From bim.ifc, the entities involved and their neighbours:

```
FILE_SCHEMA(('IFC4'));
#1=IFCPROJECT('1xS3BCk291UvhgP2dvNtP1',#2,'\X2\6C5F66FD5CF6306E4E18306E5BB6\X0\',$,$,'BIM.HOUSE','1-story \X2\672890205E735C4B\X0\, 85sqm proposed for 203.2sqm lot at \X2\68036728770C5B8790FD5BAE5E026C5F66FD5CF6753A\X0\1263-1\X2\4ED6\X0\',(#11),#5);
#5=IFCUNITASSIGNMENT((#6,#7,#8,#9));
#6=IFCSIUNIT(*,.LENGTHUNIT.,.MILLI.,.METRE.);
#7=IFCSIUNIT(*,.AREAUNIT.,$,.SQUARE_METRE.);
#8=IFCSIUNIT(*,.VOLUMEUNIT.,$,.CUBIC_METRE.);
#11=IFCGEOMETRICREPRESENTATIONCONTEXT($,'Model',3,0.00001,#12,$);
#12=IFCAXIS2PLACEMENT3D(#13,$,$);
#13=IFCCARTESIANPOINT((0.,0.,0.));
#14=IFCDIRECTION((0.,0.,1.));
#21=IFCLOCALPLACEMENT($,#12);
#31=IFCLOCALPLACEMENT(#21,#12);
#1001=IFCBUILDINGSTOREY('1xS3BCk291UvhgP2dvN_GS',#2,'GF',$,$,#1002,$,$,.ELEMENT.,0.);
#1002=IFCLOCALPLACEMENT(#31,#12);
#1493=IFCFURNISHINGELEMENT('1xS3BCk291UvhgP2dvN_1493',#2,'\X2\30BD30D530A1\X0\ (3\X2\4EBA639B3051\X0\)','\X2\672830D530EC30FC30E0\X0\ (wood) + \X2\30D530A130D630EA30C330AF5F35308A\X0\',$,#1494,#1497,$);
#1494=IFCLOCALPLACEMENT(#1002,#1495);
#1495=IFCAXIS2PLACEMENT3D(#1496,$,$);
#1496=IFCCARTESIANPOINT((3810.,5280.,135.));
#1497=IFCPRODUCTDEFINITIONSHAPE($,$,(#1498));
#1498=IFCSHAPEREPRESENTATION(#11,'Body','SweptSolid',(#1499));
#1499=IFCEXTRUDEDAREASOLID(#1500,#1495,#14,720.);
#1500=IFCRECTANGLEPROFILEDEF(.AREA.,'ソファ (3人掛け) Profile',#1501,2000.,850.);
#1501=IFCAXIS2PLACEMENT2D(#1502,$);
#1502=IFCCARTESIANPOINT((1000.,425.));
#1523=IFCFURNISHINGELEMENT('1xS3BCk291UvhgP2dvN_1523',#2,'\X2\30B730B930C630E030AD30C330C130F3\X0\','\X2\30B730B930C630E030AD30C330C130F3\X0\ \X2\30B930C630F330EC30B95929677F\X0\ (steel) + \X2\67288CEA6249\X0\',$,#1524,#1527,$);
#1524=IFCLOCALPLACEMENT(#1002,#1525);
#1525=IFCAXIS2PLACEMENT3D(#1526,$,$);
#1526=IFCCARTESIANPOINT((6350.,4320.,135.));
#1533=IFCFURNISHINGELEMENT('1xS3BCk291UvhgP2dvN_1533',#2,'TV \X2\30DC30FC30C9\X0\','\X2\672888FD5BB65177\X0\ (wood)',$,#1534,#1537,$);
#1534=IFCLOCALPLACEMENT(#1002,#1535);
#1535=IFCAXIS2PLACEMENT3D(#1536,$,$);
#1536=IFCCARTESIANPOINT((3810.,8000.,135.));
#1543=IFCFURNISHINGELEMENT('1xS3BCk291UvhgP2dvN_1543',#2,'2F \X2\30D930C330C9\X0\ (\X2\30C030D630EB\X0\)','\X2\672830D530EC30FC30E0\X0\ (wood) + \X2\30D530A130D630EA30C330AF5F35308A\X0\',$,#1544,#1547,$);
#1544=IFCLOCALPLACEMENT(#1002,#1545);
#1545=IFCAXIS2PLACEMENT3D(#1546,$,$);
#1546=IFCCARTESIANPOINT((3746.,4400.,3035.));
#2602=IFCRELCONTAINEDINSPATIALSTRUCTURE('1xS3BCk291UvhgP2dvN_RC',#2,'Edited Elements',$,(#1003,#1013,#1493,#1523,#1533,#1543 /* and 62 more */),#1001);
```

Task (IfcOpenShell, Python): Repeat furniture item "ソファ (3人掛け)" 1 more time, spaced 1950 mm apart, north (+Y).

```python
import numpy as np
import ifcopenshell
import ifcopenshell.api.geometry
import ifcopenshell.api.root
import ifcopenshell.util.element
import ifcopenshell.util.placement
import ifcopenshell.util.unit

model = ifcopenshell.open("bim.ifc")
unit_scale = ifcopenshell.util.unit.calculate_unit_scale(model)


def reuse_history(source, copy):
    """copy_class also copies each property set's owner history, people and application; keep the originals."""
    for rel in copy.IsDefinedBy:
        if rel.is_a("IfcRelDefinesByProperties") and (history := rel.RelatingPropertyDefinition.OwnerHistory):
            rel.RelatingPropertyDefinition.OwnerHistory = source.OwnerHistory
            ifcopenshell.util.element.remove_deep2(model, history)


source = model.by_id(1493)
base = ifcopenshell.util.placement.get_local_placement(source.ObjectPlacement)
step = np.array([0.0, 1.0, 0.0]) * 1.95 / unit_scale

for i in range(1, 2):
    copy = ifcopenshell.api.root.copy_class(model, product=source)
    copy.Representation = ifcopenshell.util.element.copy_deep(
        model, source.Representation, exclude=["IfcGeometricRepresentationContext", "IfcRepresentationMap"]
    )
    reuse_history(source, copy)
    matrix = base.copy()
    matrix[:3, 3] += i * step
    print("added at", matrix[:3, 3].round(3) + 0.0)
    ifcopenshell.api.geometry.edit_object_placement(model, product=copy, matrix=matrix, is_si=False)

model.write("bim-out.ifc")
```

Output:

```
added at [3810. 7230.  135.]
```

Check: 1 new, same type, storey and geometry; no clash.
